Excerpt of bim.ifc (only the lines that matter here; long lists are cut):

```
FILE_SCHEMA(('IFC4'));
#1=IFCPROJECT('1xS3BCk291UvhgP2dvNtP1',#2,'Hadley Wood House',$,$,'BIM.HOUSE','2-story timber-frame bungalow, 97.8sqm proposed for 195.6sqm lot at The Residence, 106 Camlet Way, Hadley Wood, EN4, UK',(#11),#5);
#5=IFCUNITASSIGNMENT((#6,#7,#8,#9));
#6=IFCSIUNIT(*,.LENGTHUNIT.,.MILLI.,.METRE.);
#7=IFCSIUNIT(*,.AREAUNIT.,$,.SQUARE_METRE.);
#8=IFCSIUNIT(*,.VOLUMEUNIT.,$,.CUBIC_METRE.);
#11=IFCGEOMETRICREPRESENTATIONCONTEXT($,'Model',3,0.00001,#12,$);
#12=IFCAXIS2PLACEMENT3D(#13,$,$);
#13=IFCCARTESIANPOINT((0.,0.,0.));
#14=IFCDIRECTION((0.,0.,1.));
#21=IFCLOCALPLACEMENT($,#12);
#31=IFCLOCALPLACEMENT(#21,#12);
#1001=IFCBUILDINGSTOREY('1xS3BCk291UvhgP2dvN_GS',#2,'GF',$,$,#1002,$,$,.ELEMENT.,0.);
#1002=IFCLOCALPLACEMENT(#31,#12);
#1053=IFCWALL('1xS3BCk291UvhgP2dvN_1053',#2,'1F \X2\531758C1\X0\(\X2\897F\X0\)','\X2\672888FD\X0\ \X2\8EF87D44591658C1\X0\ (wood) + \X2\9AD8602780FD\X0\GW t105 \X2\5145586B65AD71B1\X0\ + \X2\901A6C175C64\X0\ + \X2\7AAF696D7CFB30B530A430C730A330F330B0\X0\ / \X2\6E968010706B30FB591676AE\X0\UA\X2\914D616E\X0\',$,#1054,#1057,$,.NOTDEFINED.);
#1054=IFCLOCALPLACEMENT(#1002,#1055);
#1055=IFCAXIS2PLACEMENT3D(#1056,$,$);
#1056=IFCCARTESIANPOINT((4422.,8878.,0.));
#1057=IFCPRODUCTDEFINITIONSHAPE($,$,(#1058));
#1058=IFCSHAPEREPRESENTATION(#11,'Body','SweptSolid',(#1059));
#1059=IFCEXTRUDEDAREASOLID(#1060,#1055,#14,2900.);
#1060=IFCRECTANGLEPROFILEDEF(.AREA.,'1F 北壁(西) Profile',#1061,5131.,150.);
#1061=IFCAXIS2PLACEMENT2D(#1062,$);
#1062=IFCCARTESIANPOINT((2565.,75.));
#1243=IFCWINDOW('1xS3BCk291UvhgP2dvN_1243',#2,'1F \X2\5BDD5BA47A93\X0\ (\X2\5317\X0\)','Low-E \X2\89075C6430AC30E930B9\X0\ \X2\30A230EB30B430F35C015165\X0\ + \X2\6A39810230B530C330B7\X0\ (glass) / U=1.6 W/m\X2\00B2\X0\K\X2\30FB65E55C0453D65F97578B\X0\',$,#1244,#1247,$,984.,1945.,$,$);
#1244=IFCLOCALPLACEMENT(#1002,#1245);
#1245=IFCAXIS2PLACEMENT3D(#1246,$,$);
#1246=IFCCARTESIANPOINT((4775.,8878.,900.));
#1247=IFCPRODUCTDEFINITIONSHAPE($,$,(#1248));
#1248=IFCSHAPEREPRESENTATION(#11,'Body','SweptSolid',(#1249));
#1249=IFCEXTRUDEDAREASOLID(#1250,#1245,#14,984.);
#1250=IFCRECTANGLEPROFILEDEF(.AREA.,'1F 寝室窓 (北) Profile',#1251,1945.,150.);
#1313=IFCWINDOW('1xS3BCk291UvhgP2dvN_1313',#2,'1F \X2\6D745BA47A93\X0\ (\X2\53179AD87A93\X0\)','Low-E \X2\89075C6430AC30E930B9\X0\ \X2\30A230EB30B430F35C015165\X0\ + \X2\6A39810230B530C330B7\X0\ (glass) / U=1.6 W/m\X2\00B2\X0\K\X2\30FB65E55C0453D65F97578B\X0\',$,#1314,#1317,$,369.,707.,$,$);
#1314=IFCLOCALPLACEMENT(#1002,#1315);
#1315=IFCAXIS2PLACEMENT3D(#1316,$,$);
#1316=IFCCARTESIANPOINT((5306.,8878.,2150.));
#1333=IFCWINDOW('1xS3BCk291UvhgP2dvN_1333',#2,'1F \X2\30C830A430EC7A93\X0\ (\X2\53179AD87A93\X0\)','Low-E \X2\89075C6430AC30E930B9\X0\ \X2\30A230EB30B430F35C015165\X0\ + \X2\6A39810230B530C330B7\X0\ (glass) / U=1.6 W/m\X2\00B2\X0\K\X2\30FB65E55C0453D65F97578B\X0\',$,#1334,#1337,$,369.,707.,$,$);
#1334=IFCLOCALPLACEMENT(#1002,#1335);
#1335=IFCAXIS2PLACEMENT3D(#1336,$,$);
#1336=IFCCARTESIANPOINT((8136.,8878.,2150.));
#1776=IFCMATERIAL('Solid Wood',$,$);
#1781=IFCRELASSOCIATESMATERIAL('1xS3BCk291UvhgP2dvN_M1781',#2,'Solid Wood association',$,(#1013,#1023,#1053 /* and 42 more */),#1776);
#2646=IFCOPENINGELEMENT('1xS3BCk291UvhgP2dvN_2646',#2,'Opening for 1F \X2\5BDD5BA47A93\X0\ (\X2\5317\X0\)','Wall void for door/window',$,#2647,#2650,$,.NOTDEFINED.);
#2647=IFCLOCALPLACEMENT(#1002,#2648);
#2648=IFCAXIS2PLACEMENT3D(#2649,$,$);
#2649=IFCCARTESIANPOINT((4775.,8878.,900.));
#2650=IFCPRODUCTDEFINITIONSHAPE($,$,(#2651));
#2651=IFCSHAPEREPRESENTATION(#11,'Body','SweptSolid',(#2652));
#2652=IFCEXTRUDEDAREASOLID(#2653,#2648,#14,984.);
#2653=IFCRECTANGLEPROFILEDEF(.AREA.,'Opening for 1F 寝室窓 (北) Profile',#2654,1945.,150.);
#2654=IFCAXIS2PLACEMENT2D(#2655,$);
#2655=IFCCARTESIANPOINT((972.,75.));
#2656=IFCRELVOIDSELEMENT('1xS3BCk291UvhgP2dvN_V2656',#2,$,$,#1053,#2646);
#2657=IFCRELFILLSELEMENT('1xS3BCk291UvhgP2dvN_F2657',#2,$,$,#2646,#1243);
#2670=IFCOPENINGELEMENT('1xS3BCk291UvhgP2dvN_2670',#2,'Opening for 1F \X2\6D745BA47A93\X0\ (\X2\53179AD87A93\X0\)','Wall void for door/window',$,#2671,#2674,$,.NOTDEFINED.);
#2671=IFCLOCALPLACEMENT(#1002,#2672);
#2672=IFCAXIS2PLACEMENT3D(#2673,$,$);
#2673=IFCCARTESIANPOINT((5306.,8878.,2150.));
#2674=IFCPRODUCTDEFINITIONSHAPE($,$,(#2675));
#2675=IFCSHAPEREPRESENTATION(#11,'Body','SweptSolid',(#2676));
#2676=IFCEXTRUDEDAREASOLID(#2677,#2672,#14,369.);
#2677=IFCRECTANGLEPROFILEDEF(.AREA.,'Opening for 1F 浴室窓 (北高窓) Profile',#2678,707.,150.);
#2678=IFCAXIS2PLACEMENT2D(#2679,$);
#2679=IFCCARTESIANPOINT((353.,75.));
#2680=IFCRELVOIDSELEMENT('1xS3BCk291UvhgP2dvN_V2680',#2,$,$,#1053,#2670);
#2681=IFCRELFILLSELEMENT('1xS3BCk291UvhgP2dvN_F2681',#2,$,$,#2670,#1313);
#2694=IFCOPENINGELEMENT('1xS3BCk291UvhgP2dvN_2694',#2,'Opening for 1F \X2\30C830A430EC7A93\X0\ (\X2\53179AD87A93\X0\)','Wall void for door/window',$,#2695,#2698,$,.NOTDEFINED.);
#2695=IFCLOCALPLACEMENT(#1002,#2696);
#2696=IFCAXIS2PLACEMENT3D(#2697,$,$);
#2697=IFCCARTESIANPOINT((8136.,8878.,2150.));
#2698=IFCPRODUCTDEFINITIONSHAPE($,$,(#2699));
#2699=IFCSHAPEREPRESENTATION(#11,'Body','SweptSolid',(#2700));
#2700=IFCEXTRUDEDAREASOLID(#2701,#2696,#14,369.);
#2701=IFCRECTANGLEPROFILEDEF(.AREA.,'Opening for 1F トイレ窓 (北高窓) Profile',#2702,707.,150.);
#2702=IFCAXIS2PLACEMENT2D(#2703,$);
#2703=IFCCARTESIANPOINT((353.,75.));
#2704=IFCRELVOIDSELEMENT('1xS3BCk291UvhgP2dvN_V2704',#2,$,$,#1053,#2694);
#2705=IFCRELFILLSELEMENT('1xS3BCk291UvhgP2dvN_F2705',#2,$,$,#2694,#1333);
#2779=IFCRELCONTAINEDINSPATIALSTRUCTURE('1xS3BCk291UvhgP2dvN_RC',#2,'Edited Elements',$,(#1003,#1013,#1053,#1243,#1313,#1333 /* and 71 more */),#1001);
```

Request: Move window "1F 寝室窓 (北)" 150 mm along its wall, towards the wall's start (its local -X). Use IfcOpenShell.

```python
import ifcopenshell
import ifcopenshell.api.geometry
import ifcopenshell.util.placement
import ifcopenshell.util.unit

model = ifcopenshell.open("bim.ifc")
unit_scale = ifcopenshell.util.unit.calculate_unit_scale(model)

window = model.by_guid("1xS3BCk291UvhgP2dvN_1243")
opening = window.FillsVoids[0].RelatingOpeningElement
wall = opening.VoidsElements[0].RelatingBuildingElement

wall_matrix = ifcopenshell.util.placement.get_local_placement(wall.ObjectPlacement)
shift = wall_matrix[:3, 0] * -0.15 / unit_scale
before = ifcopenshell.util.placement.get_local_placement(window.ObjectPlacement)[:3, 3].copy()

# The window is not placed relative to its opening, so move both.
for product in (opening, window):
    matrix = ifcopenshell.util.placement.get_local_placement(product.ObjectPlacement)
    matrix[:3, 3] += shift
    ifcopenshell.api.geometry.edit_object_placement(model, product=product, matrix=matrix, is_si=False)

after = ifcopenshell.util.placement.get_local_placement(window.ObjectPlacement)[:3, 3]
print("window moved by", (after - before).round(3) + 0.0)

model.write("bim_updated.ifc")
```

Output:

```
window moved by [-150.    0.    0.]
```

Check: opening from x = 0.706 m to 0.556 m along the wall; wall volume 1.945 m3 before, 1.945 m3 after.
